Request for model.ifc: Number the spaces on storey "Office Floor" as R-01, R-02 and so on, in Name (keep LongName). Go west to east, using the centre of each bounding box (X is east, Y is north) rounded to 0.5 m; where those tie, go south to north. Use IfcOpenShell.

First a look at what the model holds.

```python
import ifcopenshell
import ifcopenshell.util.element
import ifcopenshell.util.placement

model = ifcopenshell.open("model.ifc")
print(model.schema)
storey = next(s for s in model.by_type("IfcBuildingStorey") if s.Name == "Office Floor")
spaces = [e for e in ifcopenshell.util.element.get_decomposition(storey) if e.is_a("IfcSpace")]
for e in sorted(spaces, key=lambda e: e.id()):
    origin = ifcopenshell.util.placement.get_local_placement(e.ObjectPlacement)[:3, 3]
    print(e.id(), e.Name, e.LongName, origin.round(2) + 0.0, sep=" | ")
```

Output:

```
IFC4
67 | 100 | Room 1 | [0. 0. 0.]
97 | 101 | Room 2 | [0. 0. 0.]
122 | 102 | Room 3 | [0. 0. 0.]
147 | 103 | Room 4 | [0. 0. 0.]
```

```python
import ifcopenshell
import ifcopenshell.geom
import ifcopenshell.util.element
import ifcopenshell.util.shape

model = ifcopenshell.open("model.ifc")
settings = ifcopenshell.geom.settings()
settings.set("use-world-coords", True)


def centre(element):
    shape = ifcopenshell.geom.create_shape(settings, element)
    return ifcopenshell.util.shape.get_bbox_centroid(shape.geometry)


storey = next(s for s in model.by_type("IfcBuildingStorey") if s.Name == "Office Floor")
spaces = [e for e in ifcopenshell.util.element.get_decomposition(storey) if e.is_a("IfcSpace")]

# Insertion points can sit at a corner or the storey origin, so sort by the geometry (in metres).
centres = {e: centre(e) for e in spaces}
spaces.sort(key=lambda e: (round(centres[e][0] / 0.5), centres[e][1]))

for i, e in enumerate(spaces, start=1):
    number = f"R-{i:02d}"
    e.Name = number
    print(e.id(), number)

model.write("model_edited.ifc")
```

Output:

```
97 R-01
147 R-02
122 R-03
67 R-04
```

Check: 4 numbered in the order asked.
